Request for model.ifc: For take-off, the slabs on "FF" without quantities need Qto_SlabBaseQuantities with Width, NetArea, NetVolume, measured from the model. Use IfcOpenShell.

First a look at what the model holds.

```python
import ifcopenshell
import ifcopenshell.util.element
import ifcopenshell.util.unit

model = ifcopenshell.open("model.ifc")
print(model.schema)
for unit_type in ("LENGTHUNIT", "AREAUNIT", "VOLUMEUNIT"):
    print(unit_type, ifcopenshell.util.unit.calculate_unit_scale(model, unit_type))
storey = next(s for s in model.by_type("IfcBuildingStorey") if s.Name == "FF")
slabs = [e for e in ifcopenshell.util.element.get_decomposition(storey) if e.is_a("IfcSlab")]
for e in sorted(slabs, key=lambda e: e.id()):
    print(e.id(), e.is_a(), e.Name, list(ifcopenshell.util.element.get_psets(e, qtos_only=True)), sep=" | ")
```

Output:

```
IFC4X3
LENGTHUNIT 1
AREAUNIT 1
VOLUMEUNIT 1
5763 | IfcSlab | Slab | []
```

```python
import ifcopenshell
import ifcopenshell.api.pset
import ifcopenshell.geom
import ifcopenshell.util.element
import ifcopenshell.util.shape
import ifcopenshell.util.unit

model = ifcopenshell.open("model.ifc")
unit_scale = ifcopenshell.util.unit.calculate_unit_scale(model)
area_scale = ifcopenshell.util.unit.calculate_unit_scale(model, "AREAUNIT")
volume_scale = ifcopenshell.util.unit.calculate_unit_scale(model, "VOLUMEUNIT")
settings = ifcopenshell.geom.settings()

storey = next(s for s in model.by_type("IfcBuildingStorey") if s.Name == "FF")
slabs = [e for e in ifcopenshell.util.element.get_decomposition(storey) if e.is_a("IfcSlab")]

for e in sorted(slabs, key=lambda e: e.id()):
    if ifcopenshell.util.element.get_psets(e, qtos_only=True, should_inherit=False):
        continue
    # Geometry comes back in metres, in the element's own axes.
    shape = ifcopenshell.geom.create_shape(settings, e)
    values = {
        "Width": ifcopenshell.util.shape.get_z(shape.geometry) / unit_scale,
        "NetArea": ifcopenshell.util.shape.get_footprint_area(shape.geometry) / area_scale,
        "NetVolume": ifcopenshell.util.shape.get_volume(shape.geometry) / volume_scale,
    }
    qto = ifcopenshell.api.pset.add_qto(model, product=e, name="Qto_SlabBaseQuantities")
    ifcopenshell.api.pset.edit_qto(model, qto=qto, properties=values)
    print(e.id(), {k: round(v, 3) for k, v in values.items()})

model.write("model_updated.ifc")
```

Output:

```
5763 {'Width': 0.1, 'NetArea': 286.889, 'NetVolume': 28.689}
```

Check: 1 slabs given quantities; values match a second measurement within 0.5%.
